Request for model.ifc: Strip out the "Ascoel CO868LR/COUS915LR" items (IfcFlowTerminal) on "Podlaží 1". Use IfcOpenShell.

First a look at what the model holds.

```python
import ifcopenshell
import ifcopenshell.util.element

model = ifcopenshell.open("model.ifc")
print(model.schema)
storey = next(s for s in model.by_type("IfcBuildingStorey") if s.Name == "Podlaží 1")
terminals = [e for e in ifcopenshell.util.element.get_decomposition(storey) if e.is_a("IfcFlowTerminal")]
seen = {}
for e in terminals:
    element_type = ifcopenshell.util.element.get_type(e)
    name = element_type.Name if element_type not in (None, e) else None
    seen[name] = seen.get(name, 0) + 1
for name, count in sorted(seen.items(), key=str):
    print(count, "x", name)
```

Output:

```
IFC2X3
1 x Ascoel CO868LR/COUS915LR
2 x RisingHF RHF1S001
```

```python
import ifcopenshell
import ifcopenshell.api.root
import ifcopenshell.util.element

model = ifcopenshell.open("model.ifc")

storey = next(s for s in model.by_type("IfcBuildingStorey") if s.Name == "Podlaží 1")
terminals = [e for e in ifcopenshell.util.element.get_decomposition(storey) if e.is_a("IfcFlowTerminal")]
targets = [e for e in terminals if (t := ifcopenshell.util.element.get_type(e)) not in (None, e) and t.Name == "Ascoel CO868LR/COUS915LR"]

for e in targets:
    ifcopenshell.api.root.remove_product(model, product=e)
print(len(targets), "removed")

model.write("model-out.ifc")
```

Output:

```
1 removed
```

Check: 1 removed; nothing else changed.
